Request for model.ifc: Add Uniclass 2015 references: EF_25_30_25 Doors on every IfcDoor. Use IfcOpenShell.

First a look at what the model holds.

```python
import ifcopenshell

model = ifcopenshell.open("model.ifc")
print(model.schema)
print("classifications:", [c.Name for c in model.by_type("IfcClassification")])
for ifc_class in ("IfcDoor", "IfcRoof", "IfcStair", "IfcWall", "IfcWindow"):
    print(ifc_class, len(model.by_type(ifc_class)))
```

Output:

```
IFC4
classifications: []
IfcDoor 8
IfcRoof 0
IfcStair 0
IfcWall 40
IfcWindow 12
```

```python
import ifcopenshell
import ifcopenshell.api.classification

model = ifcopenshell.open("model.ifc")

system = ifcopenshell.api.classification.add_classification(model, classification="Uniclass 2015")

codes = {
    "IfcDoor": ("EF_25_30_25", "Doors"),
}
for ifc_class, (code, name) in codes.items():
    products = model.by_type(ifc_class)
    ifcopenshell.api.classification.add_reference(
        model, products=products, classification=system, identification=code, name=name
    )
    print(code, len(products))

model.write("model_updated.ifc")
```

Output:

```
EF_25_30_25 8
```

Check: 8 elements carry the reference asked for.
